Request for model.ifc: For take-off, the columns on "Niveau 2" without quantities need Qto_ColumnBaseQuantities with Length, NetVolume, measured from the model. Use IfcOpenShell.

First a look at what the model holds.

```python
import ifcopenshell
import ifcopenshell.util.element
import ifcopenshell.util.unit

model = ifcopenshell.open("model.ifc")
print(model.schema)
for unit_type in ("LENGTHUNIT", "AREAUNIT", "VOLUMEUNIT"):
    print(unit_type, ifcopenshell.util.unit.calculate_unit_scale(model, unit_type))
storey = next(s for s in model.by_type("IfcBuildingStorey") if s.Name == "Niveau 2")
columns = [e for e in ifcopenshell.util.element.get_decomposition(storey) if e.is_a("IfcColumn")]
for e in sorted(columns, key=lambda e: e.id()):
    print(e.id(), e.is_a(), e.Name, list(ifcopenshell.util.element.get_psets(e, qtos_only=True)), sep=" | ")
```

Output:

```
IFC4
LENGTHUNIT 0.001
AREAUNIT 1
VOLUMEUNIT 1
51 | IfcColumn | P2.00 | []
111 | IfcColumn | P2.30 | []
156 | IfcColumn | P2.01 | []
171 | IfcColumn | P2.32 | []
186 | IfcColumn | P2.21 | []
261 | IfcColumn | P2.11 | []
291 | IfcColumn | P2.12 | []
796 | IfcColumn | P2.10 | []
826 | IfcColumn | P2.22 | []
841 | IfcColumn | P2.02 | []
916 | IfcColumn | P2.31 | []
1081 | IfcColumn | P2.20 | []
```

```python
import ifcopenshell
import ifcopenshell.api.pset
import ifcopenshell.geom
import ifcopenshell.util.element
import ifcopenshell.util.shape
import ifcopenshell.util.unit

model = ifcopenshell.open("model.ifc")
unit_scale = ifcopenshell.util.unit.calculate_unit_scale(model)
volume_scale = ifcopenshell.util.unit.calculate_unit_scale(model, "VOLUMEUNIT")
settings = ifcopenshell.geom.settings()

storey = next(s for s in model.by_type("IfcBuildingStorey") if s.Name == "Niveau 2")
columns = [e for e in ifcopenshell.util.element.get_decomposition(storey) if e.is_a("IfcColumn")]

for e in sorted(columns, key=lambda e: e.id()):
    if ifcopenshell.util.element.get_psets(e, qtos_only=True, should_inherit=False):
        continue
    # Geometry comes back in metres, in the element's own axes.
    shape = ifcopenshell.geom.create_shape(settings, e)
    values = {
        "Length": ifcopenshell.util.shape.get_z(shape.geometry) / unit_scale,
        "NetVolume": ifcopenshell.util.shape.get_volume(shape.geometry) / volume_scale,
    }
    qto = ifcopenshell.api.pset.add_qto(model, product=e, name="Qto_ColumnBaseQuantities")
    ifcopenshell.api.pset.edit_qto(model, qto=qto, properties=values)
    print(e.id(), {k: round(v, 3) for k, v in values.items()})

model.write("model-out.ifc")
```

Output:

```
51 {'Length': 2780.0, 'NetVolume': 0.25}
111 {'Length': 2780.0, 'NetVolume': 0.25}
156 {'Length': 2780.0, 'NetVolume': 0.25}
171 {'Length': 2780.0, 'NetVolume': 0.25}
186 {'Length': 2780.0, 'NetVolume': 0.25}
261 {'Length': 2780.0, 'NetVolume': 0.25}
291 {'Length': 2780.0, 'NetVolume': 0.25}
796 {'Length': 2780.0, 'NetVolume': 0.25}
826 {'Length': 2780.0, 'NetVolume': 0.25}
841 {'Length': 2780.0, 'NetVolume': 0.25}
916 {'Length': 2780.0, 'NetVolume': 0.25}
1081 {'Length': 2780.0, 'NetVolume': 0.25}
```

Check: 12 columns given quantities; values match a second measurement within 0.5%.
